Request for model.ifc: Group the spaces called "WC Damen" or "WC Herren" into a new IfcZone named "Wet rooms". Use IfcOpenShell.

First a look at what the model holds.

```python
import ifcopenshell

model = ifcopenshell.open("model.ifc")
print(model.schema)
seen = {}
for space in model.by_type("IfcSpace"):
    seen[space.LongName] = seen.get(space.LongName, 0) + 1
for name, count in sorted(seen.items(), key=str):
    print(count, "x", name)
print("zones:", [z.Name for z in model.by_type("IfcZone")][:20])
```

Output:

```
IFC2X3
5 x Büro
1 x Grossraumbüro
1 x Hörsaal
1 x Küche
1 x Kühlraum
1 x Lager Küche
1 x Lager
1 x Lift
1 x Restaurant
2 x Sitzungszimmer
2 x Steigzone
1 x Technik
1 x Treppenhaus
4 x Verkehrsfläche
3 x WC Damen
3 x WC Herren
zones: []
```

```python
import ifcopenshell
import ifcopenshell.api.group
import ifcopenshell.api.root

model = ifcopenshell.open("model.ifc")

names = {"WC Damen", "WC Herren"}
spaces = [s for s in model.by_type("IfcSpace") if s.LongName in names]

zone = ifcopenshell.api.root.create_entity(model, ifc_class="IfcZone", name="Wet rooms")
ifcopenshell.api.group.assign_group(model, products=spaces, group=zone)
print(len(spaces), "spaces in", zone.Name)

model.write("model_v2.ifc")
```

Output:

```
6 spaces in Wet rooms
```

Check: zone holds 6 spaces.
